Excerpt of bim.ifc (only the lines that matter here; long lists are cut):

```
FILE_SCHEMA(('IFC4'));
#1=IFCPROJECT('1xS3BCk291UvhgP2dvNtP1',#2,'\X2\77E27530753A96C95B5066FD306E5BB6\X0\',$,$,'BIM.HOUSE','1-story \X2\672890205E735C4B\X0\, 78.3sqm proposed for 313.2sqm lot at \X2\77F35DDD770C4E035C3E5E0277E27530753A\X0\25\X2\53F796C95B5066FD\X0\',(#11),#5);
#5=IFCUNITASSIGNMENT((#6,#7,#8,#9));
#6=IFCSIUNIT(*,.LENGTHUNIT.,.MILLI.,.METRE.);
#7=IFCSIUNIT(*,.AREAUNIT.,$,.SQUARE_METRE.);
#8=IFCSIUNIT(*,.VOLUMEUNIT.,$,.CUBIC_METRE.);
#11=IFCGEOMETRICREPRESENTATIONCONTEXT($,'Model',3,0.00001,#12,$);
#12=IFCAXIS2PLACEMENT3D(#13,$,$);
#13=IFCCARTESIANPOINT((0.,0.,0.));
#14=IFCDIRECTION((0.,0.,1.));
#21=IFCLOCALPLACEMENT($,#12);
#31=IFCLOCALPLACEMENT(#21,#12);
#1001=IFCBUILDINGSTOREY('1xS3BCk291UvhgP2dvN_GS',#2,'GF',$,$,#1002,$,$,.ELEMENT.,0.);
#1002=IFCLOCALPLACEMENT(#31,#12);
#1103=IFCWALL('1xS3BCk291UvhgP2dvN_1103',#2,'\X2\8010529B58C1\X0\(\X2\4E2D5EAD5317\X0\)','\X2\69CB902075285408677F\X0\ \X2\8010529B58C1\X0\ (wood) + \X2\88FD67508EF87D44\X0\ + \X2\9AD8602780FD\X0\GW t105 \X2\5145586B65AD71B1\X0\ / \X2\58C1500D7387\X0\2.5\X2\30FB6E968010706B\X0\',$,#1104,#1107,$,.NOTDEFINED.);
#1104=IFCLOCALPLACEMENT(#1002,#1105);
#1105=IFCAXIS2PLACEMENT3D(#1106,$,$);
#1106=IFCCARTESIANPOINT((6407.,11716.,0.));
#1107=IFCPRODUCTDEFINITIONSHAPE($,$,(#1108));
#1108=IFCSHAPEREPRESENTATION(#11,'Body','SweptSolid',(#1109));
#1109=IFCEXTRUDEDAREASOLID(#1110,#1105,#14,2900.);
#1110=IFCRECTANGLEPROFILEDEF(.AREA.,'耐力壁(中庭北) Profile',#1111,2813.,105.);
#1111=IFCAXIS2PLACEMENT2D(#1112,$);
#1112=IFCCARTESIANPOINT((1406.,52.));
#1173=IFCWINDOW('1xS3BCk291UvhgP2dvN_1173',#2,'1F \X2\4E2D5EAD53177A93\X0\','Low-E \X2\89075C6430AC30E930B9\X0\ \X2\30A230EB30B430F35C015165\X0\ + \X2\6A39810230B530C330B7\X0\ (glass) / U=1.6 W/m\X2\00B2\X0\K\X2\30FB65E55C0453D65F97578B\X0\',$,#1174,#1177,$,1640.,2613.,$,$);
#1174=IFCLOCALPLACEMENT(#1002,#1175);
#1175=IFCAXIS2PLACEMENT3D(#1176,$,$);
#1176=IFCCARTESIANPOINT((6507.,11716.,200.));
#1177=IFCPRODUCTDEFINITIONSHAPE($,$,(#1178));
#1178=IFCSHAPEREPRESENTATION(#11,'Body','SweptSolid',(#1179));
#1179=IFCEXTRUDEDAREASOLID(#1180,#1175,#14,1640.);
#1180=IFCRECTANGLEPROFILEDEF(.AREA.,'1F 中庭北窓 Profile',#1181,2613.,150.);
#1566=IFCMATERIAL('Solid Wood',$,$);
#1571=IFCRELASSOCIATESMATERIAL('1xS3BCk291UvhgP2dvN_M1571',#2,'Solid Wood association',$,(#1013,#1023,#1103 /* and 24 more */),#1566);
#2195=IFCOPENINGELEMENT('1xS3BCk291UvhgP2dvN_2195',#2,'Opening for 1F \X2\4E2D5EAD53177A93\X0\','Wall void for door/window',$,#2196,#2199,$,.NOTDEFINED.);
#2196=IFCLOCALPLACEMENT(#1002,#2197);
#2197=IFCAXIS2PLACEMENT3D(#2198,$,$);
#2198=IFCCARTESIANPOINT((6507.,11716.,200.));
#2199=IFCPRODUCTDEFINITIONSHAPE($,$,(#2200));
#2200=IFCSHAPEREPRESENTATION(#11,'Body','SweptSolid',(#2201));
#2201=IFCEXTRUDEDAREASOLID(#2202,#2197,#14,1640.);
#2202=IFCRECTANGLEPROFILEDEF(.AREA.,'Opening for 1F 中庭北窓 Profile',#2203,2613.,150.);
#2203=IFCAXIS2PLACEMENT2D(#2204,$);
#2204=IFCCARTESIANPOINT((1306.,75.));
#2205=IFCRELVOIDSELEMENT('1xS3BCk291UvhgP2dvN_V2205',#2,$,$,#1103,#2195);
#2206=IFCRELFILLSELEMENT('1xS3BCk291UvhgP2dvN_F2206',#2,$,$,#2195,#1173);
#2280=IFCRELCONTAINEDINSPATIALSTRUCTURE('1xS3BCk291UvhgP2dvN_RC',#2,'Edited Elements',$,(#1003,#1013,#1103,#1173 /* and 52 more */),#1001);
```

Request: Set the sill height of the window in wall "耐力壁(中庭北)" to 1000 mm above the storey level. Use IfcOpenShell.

```python
import numpy as np
import ifcopenshell
import ifcopenshell.api.geometry
import ifcopenshell.geom
import ifcopenshell.util.element
import ifcopenshell.util.placement
import ifcopenshell.util.shape
import ifcopenshell.util.unit

model = ifcopenshell.open("bim.ifc")
unit_scale = ifcopenshell.util.unit.calculate_unit_scale(model)

window = model.by_guid("1xS3BCk291UvhgP2dvN_1173")
opening = window.FillsVoids[0].RelatingOpeningElement
storey = ifcopenshell.util.element.get_container(window, ifc_class="IfcBuildingStorey")
level = ifcopenshell.util.placement.get_local_placement(storey.ObjectPlacement)[2, 3]

# The opening's origin need not be at the sill, so measure its lowest point.
shape = ifcopenshell.geom.create_shape(ifcopenshell.geom.settings(), opening)
bottom = ifcopenshell.util.shape.get_shape_bottom_elevation(shape, shape.geometry) / unit_scale
dz = level + 1 / unit_scale - bottom

shift = np.array([0.0, 0.0, dz])
# The window is not placed relative to its opening, so move both.
for product in (opening, window):
    matrix = ifcopenshell.util.placement.get_local_placement(product.ObjectPlacement)
    matrix[:3, 3] += shift
    ifcopenshell.api.geometry.edit_object_placement(model, product=product, matrix=matrix, is_si=False)

print(f"moved by {dz * unit_scale:+.3f} m")

model.write("bim_edited.ifc")
```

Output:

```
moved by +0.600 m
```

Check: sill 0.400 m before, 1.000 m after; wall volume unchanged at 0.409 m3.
